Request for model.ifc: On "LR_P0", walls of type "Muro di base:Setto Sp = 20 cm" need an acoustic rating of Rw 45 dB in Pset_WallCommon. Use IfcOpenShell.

First a look at what the model holds.

```python
import ifcopenshell
import ifcopenshell.util.element

model = ifcopenshell.open("model.ifc")
print(model.schema)
storey = next(s for s in model.by_type("IfcBuildingStorey") if s.Name == "LR_P0")
walls = [e for e in ifcopenshell.util.element.get_decomposition(storey) if e.is_a("IfcWall")]
seen = {}
for e in walls:
    element_type = ifcopenshell.util.element.get_type(e)
    key = (element_type.Name if element_type != e and element_type else None, ifcopenshell.util.element.get_pset(e, "Pset_WallCommon", "AcousticRating"))
    seen[key] = seen.get(key, 0) + 1
for (name, value), count in sorted(seen.items(), key=str):
    print(count, "x", name, "|", value)
```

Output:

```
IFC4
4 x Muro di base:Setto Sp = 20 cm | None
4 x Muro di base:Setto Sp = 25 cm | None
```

```python
import ifcopenshell
import ifcopenshell.api.pset
import ifcopenshell.util.element

model = ifcopenshell.open("model.ifc")

storey = next(s for s in model.by_type("IfcBuildingStorey") if s.Name == "LR_P0")
walls = [e for e in ifcopenshell.util.element.get_decomposition(storey) if e.is_a("IfcWall")]

count = 0
for e in walls:
    element_type = ifcopenshell.util.element.get_type(e)
    if element_type in (None, e) or element_type.Name != "Muro di base:Setto Sp = 20 cm":
        continue
    # add_pset returns the element's existing set when there is one.
    pset = ifcopenshell.api.pset.add_pset(model, product=e, name="Pset_WallCommon")
    ifcopenshell.api.pset.edit_pset(model, pset=pset, properties={"AcousticRating": "Rw 45 dB"})
    count += 1

print(count, "walls updated")

model.write("model_v2.ifc")
```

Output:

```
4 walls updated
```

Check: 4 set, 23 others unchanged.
